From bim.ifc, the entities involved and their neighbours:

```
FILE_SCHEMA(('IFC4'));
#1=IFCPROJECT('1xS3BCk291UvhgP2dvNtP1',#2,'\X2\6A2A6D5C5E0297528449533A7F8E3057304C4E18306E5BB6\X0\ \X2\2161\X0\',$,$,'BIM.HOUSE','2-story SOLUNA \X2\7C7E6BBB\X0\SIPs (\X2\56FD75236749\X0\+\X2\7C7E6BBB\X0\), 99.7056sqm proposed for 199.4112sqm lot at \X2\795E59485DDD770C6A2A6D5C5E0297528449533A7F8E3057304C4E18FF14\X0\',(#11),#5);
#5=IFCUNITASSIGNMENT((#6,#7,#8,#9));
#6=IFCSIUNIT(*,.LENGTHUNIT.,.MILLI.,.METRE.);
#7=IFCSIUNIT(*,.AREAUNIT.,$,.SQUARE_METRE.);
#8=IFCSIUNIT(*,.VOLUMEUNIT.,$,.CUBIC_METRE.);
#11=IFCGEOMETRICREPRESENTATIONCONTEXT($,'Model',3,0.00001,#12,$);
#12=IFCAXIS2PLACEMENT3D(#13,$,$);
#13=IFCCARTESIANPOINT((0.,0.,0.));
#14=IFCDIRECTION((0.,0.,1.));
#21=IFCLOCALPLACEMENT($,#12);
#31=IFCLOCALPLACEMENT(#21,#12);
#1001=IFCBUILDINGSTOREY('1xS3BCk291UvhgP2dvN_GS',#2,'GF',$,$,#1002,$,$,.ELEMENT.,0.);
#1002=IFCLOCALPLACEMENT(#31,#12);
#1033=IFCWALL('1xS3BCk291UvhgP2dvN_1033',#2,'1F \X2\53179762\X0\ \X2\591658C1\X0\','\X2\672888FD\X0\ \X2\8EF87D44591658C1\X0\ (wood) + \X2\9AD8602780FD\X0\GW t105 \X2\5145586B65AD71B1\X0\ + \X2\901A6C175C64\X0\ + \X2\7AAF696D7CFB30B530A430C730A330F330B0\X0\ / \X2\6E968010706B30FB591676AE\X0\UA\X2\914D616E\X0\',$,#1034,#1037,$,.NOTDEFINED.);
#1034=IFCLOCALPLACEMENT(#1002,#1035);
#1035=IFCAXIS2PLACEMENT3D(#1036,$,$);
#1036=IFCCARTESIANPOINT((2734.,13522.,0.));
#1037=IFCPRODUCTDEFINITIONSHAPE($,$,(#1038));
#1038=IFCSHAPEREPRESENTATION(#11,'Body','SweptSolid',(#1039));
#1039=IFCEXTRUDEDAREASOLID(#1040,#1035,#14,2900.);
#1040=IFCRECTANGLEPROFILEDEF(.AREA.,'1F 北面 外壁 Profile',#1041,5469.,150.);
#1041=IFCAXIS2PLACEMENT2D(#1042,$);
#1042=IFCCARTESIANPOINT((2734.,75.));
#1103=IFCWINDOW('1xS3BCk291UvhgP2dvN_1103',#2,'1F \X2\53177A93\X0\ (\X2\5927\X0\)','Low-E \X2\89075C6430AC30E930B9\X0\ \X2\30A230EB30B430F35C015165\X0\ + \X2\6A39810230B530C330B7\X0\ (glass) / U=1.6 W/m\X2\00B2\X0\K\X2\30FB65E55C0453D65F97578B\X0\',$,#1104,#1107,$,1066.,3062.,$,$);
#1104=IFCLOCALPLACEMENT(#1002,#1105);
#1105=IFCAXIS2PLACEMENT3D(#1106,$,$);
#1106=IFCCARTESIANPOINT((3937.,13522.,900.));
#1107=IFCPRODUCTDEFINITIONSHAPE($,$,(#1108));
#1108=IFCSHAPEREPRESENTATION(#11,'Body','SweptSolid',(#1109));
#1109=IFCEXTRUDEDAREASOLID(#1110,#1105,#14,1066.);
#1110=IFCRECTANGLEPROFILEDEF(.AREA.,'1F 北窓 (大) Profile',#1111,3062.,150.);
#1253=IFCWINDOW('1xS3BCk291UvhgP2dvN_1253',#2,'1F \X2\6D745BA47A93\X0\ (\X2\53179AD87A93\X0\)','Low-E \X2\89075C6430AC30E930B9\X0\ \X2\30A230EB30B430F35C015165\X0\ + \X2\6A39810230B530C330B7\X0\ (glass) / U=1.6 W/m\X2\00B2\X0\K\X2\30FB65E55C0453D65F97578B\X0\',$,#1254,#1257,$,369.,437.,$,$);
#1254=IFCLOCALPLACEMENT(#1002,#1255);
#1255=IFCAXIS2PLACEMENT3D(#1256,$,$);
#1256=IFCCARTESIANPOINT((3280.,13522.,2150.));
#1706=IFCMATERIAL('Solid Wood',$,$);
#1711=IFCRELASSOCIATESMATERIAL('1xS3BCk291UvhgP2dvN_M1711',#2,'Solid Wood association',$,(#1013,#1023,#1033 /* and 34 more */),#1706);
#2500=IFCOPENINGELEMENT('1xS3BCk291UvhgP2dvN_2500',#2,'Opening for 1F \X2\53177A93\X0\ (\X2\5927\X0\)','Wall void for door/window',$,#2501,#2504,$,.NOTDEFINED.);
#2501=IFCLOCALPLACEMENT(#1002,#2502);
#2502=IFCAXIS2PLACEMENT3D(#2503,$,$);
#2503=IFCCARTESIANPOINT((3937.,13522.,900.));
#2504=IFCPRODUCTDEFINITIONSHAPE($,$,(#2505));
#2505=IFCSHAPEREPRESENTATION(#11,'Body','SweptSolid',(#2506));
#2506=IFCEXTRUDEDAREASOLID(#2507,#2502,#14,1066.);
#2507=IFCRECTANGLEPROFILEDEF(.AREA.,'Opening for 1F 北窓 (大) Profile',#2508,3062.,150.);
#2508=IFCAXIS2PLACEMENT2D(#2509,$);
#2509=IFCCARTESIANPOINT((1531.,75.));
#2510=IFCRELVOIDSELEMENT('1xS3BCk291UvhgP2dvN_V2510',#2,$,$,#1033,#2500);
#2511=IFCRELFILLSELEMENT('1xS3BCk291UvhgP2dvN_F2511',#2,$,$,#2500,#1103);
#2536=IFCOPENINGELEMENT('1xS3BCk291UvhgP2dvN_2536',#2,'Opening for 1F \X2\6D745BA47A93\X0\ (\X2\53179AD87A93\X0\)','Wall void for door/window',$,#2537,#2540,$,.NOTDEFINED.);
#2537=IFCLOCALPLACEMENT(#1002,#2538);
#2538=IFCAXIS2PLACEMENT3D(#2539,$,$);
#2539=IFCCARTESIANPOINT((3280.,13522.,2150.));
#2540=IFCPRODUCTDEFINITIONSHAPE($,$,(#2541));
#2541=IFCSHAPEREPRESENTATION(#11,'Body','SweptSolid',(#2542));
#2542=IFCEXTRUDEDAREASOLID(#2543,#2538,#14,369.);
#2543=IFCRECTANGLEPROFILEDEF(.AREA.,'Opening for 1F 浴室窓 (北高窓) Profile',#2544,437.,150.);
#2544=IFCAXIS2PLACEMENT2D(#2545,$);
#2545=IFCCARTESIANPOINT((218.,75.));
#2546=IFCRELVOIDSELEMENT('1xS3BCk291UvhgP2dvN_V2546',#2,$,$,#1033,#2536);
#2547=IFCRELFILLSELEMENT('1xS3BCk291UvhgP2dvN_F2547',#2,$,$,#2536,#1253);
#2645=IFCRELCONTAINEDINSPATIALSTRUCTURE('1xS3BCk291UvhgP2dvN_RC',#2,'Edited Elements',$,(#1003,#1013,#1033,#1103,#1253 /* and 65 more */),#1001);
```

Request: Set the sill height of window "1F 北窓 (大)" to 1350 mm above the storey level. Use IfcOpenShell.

```python
import numpy as np
import ifcopenshell
import ifcopenshell.api.geometry
import ifcopenshell.geom
import ifcopenshell.util.element
import ifcopenshell.util.placement
import ifcopenshell.util.shape
import ifcopenshell.util.unit

model = ifcopenshell.open("bim.ifc")
unit_scale = ifcopenshell.util.unit.calculate_unit_scale(model)

window = model.by_id(1103)
opening = window.FillsVoids[0].RelatingOpeningElement
storey = ifcopenshell.util.element.get_container(window, ifc_class="IfcBuildingStorey")
level = ifcopenshell.util.placement.get_local_placement(storey.ObjectPlacement)[2, 3]

# The opening's origin need not be at the sill, so measure its lowest point.
shape = ifcopenshell.geom.create_shape(ifcopenshell.geom.settings(), opening)
bottom = ifcopenshell.util.shape.get_shape_bottom_elevation(shape, shape.geometry) / unit_scale
dz = level + 1.35 / unit_scale - bottom

shift = np.array([0.0, 0.0, dz])
# The window is not placed relative to its opening, so move both.
for product in (opening, window):
    matrix = ifcopenshell.util.placement.get_local_placement(product.ObjectPlacement)
    matrix[:3, 3] += shift
    ifcopenshell.api.geometry.edit_object_placement(model, product=product, matrix=matrix, is_si=False)

print(f"moved by {dz * unit_scale:+.3f} m")

model.write("bim-out.ifc")
```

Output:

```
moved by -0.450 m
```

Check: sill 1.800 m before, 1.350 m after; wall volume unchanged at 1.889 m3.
